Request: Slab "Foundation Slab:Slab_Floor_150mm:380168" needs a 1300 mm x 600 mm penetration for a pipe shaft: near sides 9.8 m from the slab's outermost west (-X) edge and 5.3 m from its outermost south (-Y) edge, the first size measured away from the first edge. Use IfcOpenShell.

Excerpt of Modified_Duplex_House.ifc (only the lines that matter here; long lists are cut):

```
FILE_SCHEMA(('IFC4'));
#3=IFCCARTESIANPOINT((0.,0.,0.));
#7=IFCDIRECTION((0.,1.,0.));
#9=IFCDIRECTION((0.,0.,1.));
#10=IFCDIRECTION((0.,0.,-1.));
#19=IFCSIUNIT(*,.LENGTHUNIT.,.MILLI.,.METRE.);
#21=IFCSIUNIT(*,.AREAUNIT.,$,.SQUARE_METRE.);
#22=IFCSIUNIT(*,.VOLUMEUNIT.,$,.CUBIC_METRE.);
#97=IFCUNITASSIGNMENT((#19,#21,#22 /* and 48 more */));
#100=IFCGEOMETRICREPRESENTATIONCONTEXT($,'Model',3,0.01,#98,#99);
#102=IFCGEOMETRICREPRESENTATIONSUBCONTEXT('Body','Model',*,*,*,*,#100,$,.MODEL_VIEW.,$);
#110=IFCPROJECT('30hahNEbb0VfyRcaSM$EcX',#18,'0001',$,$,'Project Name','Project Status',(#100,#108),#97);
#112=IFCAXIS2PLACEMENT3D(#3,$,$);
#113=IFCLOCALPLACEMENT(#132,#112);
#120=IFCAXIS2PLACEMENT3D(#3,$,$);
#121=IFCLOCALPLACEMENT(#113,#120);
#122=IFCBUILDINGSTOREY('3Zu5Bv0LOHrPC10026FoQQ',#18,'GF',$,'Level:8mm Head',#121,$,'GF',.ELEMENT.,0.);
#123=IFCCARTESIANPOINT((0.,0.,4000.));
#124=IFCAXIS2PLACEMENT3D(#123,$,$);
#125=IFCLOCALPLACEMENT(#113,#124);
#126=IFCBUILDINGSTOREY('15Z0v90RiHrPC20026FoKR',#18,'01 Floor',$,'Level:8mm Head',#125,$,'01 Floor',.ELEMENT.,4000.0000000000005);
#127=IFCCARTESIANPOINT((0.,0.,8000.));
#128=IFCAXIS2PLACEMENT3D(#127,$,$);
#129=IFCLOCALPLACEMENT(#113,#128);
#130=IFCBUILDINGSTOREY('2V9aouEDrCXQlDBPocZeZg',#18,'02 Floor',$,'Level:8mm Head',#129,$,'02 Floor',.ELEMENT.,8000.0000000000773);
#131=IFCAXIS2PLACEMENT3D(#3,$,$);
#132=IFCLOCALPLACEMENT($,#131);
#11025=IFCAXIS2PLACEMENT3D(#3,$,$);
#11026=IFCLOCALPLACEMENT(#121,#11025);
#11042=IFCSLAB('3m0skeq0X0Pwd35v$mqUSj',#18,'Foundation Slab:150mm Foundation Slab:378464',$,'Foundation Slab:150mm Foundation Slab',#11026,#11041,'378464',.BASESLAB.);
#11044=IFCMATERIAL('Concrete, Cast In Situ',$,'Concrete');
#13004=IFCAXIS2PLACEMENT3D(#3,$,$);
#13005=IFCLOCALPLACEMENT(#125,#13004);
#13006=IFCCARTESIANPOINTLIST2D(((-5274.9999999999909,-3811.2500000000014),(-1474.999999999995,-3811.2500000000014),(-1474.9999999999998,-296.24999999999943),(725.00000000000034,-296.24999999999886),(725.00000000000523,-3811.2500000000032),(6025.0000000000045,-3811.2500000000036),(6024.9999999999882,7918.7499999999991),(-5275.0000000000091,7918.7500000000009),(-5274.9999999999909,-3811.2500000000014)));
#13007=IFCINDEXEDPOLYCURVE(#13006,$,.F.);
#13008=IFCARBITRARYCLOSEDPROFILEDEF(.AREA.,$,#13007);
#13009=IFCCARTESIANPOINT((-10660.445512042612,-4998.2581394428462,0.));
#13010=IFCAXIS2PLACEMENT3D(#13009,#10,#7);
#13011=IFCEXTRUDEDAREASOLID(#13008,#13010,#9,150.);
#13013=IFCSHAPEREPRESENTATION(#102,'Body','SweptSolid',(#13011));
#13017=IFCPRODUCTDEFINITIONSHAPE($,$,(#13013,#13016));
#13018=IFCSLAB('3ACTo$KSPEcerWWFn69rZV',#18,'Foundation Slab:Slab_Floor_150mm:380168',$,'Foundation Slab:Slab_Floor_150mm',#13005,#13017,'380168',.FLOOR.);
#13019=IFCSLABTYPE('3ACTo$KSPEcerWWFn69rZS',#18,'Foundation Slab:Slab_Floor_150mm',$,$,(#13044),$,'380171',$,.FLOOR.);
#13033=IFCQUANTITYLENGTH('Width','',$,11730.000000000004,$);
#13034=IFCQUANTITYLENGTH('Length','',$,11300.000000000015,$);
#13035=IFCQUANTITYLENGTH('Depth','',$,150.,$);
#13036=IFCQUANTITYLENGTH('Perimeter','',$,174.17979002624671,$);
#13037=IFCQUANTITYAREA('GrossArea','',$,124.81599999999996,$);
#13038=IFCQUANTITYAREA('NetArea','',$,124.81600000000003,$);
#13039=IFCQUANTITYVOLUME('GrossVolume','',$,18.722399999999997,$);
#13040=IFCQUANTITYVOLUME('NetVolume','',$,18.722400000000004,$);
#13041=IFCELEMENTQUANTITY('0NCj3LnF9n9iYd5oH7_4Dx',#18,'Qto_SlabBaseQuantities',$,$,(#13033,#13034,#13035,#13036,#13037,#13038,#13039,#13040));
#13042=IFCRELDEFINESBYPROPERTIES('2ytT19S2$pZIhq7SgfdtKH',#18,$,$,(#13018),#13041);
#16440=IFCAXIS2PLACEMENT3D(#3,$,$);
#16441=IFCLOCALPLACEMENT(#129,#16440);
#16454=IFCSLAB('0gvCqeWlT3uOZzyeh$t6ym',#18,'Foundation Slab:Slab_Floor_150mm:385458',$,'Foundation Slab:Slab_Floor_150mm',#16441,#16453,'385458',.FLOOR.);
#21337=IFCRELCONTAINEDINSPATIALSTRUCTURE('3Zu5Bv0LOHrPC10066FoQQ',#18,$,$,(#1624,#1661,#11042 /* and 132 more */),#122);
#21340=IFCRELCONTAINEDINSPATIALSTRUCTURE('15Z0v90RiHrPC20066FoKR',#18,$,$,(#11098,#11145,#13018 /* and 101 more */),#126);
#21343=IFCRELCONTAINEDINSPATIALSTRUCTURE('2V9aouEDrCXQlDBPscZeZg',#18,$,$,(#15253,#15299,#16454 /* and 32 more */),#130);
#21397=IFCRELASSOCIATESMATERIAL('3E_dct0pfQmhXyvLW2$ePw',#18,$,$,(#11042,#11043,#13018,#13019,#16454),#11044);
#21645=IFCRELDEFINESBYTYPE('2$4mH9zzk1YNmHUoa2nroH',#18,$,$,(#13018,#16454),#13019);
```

```python
import numpy as np
import ifcopenshell
import ifcopenshell.api.feature
import ifcopenshell.api.geometry
import ifcopenshell.api.pset
import ifcopenshell.api.root
import ifcopenshell.geom
import ifcopenshell.util.element
import ifcopenshell.util.placement
import ifcopenshell.util.representation
import ifcopenshell.util.shape
import ifcopenshell.util.unit

model = ifcopenshell.open("Modified_Duplex_House.ifc")
unit_scale = ifcopenshell.util.unit.calculate_unit_scale(model)
area_scale = ifcopenshell.util.unit.calculate_unit_scale(model, "AREAUNIT")
volume_scale = ifcopenshell.util.unit.calculate_unit_scale(model, "VOLUMEUNIT")
settings = ifcopenshell.geom.settings()


def volume(element):
    """Net volume in cubic metres, openings subtracted."""
    shape = ifcopenshell.geom.create_shape(settings, element)
    return ifcopenshell.util.shape.get_volume(shape.geometry)


slab = model.by_guid("3ACTo$KSPEcerWWFn69rZV")
before = volume(slab)

# Extent in the slab's own axes, in metres. The edges named are its -X and -Y sides.
slab_shape = ifcopenshell.geom.create_shape(settings, slab)
vertices = ifcopenshell.util.shape.get_vertices(slab_shape.geometry)
x_min, y_min, bottom = vertices.min(axis=0)
top = vertices[:, 2].max()

opening = ifcopenshell.api.root.create_entity(model, ifc_class="IfcOpeningElement", name="Pipe shaft opening", predefined_type="OPENING")
context = ifcopenshell.util.representation.get_context(model, "Model", "Body", "MODEL_VIEW")
width, depth = 1.3, 0.6
outline = [(0.0, 0.0), (width, 0.0), (width, depth), (0.0, depth), (0.0, 0.0)]
# Overshoot both faces by 50 mm so the cut is clean.
shape = ifcopenshell.api.geometry.add_slab_representation(
    model, context=context, depth=top - bottom + 0.1, polyline=outline
)
ifcopenshell.api.geometry.assign_representation(model, product=opening, representation=shape)

matrix = ifcopenshell.util.placement.get_local_placement(slab.ObjectPlacement)
matrix[:, 3] = matrix @ np.append(np.array([x_min + 9.8, y_min + 5.3, bottom - 0.05]) / unit_scale, 1.0)
ifcopenshell.api.geometry.edit_object_placement(model, product=opening, matrix=matrix, is_si=False)
ifcopenshell.api.feature.add_feature(model, feature=opening, element=slab)

after = volume(slab)

# Update the slab's stored quantities.
qto = model.by_id(ifcopenshell.util.element.get_pset(slab, "Qto_SlabBaseQuantities", should_inherit=False)["id"])
ifcopenshell.api.pset.edit_qto(model, qto=qto, properties={
    "NetArea": after / (top - bottom) / area_scale,
    "NetVolume": after / volume_scale,
})

print(f"slab volume {before:.3f} -> {after:.3f} m3")

model.write("Modified_Duplex_House_updated.ifc")
```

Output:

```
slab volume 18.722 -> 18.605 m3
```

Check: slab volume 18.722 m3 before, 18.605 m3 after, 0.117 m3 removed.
